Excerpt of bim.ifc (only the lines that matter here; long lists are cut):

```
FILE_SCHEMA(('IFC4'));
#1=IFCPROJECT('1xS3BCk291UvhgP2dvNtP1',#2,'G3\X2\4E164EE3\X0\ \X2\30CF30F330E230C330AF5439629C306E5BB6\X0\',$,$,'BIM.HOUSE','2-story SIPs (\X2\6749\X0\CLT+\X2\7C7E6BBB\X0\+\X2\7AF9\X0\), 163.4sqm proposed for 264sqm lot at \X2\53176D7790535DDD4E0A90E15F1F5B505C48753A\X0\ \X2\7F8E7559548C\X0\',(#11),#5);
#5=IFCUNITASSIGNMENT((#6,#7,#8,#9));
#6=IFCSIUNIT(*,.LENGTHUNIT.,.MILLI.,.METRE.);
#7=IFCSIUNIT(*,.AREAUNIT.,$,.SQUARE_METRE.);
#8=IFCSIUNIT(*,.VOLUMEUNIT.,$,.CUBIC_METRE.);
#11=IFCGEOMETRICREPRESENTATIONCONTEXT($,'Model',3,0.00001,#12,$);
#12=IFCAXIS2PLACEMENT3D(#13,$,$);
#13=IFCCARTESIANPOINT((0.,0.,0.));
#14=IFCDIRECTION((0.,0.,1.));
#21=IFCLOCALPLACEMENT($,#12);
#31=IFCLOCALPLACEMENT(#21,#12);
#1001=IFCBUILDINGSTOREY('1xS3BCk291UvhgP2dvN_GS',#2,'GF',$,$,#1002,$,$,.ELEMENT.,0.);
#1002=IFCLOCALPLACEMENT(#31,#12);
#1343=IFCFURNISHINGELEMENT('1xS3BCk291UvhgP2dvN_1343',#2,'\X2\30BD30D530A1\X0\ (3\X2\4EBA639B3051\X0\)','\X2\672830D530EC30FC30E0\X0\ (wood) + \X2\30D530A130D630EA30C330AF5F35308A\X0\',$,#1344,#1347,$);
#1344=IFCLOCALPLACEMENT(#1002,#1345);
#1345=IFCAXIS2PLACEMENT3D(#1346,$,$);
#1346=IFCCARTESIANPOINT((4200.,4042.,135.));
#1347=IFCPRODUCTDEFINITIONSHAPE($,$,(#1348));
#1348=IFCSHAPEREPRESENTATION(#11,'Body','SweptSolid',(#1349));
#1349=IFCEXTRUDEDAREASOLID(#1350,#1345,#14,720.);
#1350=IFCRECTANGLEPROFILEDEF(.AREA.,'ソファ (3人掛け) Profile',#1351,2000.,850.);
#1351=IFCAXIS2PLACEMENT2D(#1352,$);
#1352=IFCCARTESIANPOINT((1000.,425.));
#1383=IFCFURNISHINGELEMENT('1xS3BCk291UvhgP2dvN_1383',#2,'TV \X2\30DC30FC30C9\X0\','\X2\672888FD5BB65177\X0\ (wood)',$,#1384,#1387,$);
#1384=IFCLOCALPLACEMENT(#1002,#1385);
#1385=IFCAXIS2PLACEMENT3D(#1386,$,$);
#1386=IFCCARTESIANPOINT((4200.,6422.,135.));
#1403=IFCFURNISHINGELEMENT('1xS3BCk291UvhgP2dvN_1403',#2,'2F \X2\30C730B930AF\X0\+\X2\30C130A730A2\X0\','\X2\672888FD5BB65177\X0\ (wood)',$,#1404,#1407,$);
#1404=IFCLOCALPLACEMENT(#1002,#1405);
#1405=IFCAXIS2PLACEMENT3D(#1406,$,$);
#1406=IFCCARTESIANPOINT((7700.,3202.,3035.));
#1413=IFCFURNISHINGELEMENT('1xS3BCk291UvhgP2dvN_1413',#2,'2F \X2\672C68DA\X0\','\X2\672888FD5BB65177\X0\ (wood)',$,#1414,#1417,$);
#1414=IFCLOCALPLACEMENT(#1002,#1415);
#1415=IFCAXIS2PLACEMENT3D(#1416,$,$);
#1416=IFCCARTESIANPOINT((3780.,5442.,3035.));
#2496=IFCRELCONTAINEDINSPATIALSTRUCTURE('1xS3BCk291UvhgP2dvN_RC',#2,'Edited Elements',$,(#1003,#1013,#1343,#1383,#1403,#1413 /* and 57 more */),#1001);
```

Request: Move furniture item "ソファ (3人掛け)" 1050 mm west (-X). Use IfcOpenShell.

```python
import ifcopenshell
import ifcopenshell.api.geometry
import ifcopenshell.util.placement

model = ifcopenshell.open("bim.ifc")

item = model.by_id(1343)
matrix = ifcopenshell.util.placement.get_local_placement(item.ObjectPlacement)
matrix[0, 3] -= 1050.0
ifcopenshell.api.geometry.edit_object_placement(model, product=item, matrix=matrix, is_si=False)

print(ifcopenshell.util.placement.get_local_placement(item.ObjectPlacement).round(3) + 0.0)

model.write("bim_edited.ifc")
```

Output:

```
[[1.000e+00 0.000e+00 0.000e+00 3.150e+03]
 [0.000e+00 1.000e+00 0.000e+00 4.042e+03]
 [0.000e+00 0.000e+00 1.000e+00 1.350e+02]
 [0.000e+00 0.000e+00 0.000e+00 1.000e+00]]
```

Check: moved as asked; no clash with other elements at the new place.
